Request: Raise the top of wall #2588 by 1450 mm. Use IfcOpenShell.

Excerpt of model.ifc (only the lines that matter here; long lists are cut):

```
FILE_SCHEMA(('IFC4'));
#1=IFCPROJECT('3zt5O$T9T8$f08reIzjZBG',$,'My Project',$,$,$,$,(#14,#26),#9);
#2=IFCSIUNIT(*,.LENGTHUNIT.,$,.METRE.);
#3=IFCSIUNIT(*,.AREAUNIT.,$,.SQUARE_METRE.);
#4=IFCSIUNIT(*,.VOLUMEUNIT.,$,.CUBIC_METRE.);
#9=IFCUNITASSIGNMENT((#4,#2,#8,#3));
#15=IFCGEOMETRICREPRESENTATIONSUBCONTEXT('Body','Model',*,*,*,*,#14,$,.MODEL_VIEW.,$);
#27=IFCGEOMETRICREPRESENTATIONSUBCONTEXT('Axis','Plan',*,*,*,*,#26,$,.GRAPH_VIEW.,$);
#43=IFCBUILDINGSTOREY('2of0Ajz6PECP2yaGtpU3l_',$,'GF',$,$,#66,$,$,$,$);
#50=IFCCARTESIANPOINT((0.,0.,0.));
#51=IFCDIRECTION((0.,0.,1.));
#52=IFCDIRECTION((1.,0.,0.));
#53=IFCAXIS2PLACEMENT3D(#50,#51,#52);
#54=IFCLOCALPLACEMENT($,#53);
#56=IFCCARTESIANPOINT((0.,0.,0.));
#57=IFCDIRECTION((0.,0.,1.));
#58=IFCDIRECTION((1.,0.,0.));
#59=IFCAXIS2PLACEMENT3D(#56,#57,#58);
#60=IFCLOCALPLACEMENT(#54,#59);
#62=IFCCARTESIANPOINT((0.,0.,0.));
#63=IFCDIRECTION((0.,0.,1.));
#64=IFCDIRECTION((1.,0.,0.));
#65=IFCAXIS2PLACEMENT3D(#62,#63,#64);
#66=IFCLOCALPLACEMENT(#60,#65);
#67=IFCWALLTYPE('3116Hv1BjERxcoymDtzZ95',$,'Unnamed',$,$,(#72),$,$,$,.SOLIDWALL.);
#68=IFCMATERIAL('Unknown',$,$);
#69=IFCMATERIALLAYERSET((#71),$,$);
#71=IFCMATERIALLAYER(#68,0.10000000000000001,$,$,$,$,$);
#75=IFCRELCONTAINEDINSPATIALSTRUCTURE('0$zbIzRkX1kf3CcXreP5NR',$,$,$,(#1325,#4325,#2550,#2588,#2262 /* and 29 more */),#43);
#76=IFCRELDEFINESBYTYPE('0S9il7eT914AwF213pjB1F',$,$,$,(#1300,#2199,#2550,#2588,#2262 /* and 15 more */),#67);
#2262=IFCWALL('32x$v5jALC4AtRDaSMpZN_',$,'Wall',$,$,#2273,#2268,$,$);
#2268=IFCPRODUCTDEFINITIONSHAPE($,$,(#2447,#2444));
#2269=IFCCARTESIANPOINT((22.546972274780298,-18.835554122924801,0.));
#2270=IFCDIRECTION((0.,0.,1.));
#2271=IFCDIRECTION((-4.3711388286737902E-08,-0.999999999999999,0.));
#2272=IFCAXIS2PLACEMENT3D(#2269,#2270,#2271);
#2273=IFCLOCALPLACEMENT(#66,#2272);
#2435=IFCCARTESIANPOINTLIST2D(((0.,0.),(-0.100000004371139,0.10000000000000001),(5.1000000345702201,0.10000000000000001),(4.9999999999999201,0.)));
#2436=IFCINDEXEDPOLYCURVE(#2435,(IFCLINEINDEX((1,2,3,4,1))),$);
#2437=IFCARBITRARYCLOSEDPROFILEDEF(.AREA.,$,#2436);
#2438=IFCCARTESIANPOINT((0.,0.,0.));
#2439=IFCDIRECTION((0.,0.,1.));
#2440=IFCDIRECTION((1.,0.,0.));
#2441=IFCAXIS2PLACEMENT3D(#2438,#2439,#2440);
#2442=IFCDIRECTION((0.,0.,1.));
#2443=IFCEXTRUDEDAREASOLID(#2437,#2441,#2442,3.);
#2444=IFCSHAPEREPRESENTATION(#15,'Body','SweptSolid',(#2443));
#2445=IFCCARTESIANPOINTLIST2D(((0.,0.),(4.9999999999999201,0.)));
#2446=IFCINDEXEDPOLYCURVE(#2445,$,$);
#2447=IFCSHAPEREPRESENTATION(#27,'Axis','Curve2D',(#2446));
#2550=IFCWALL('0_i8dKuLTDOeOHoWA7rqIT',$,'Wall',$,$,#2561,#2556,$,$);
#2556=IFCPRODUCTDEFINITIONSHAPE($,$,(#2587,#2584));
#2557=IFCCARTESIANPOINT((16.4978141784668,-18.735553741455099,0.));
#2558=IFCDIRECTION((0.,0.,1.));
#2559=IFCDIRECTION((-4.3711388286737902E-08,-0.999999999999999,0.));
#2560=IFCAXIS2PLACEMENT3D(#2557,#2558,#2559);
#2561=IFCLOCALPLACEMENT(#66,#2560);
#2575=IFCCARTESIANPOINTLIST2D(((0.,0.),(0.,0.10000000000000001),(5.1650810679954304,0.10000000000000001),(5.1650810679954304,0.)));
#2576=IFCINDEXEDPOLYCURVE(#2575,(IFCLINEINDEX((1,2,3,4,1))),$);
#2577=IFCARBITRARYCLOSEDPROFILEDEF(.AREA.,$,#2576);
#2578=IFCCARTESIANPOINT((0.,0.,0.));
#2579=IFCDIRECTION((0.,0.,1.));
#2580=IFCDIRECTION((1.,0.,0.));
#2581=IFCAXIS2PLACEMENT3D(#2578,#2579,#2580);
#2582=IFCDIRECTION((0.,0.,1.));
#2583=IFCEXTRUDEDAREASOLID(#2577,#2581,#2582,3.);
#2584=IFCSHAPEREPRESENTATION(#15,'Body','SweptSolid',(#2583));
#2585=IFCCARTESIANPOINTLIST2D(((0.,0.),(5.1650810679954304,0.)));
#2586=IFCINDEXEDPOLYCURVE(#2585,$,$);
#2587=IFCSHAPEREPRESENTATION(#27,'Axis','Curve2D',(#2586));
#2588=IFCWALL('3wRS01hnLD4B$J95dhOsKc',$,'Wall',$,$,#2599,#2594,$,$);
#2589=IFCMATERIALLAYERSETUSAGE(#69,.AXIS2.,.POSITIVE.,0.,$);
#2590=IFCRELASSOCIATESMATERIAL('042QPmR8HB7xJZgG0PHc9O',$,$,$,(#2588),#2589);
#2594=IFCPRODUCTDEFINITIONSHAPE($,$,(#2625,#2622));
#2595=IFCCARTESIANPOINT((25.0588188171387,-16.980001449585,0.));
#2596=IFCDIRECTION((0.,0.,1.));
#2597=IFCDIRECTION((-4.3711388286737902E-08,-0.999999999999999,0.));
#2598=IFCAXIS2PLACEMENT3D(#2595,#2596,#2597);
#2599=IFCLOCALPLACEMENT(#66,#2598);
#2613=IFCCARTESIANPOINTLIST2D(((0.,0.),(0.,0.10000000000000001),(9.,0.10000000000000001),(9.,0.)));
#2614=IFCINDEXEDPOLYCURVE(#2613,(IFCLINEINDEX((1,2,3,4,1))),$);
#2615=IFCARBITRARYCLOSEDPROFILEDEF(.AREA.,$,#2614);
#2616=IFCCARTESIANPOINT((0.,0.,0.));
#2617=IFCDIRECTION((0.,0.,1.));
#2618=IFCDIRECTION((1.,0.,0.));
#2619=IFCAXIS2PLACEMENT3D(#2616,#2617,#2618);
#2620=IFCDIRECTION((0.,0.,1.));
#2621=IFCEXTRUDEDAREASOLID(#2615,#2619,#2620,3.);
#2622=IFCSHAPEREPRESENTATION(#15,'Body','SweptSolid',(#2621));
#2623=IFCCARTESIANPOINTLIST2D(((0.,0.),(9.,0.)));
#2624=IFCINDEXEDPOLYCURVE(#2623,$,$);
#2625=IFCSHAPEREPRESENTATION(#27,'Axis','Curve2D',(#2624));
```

```python
import ifcopenshell
import ifcopenshell.geom
import ifcopenshell.util.representation
import ifcopenshell.util.shape
import ifcopenshell.util.unit

model = ifcopenshell.open("model.ifc")
unit_scale = ifcopenshell.util.unit.calculate_unit_scale(model)
settings = ifcopenshell.geom.settings()


def volume(element):
    """Net volume in cubic metres, openings subtracted."""
    shape = ifcopenshell.geom.create_shape(settings, element)
    return ifcopenshell.util.shape.get_volume(shape.geometry)


wall = model.by_id(2588)
before = volume(wall)

body = ifcopenshell.util.representation.get_representation(wall, "Model", "Body")
solid = body.Items[0]
old_height = solid.Depth
solid.Depth += 1.45 / unit_scale
after = volume(wall)

print(f"height {old_height:g} -> {solid.Depth:g}, volume {before:.3f} -> {after:.3f} m3")

model.write("model_rev.ifc")
```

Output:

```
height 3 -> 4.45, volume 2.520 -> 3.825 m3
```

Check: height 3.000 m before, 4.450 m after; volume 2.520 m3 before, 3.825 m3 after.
